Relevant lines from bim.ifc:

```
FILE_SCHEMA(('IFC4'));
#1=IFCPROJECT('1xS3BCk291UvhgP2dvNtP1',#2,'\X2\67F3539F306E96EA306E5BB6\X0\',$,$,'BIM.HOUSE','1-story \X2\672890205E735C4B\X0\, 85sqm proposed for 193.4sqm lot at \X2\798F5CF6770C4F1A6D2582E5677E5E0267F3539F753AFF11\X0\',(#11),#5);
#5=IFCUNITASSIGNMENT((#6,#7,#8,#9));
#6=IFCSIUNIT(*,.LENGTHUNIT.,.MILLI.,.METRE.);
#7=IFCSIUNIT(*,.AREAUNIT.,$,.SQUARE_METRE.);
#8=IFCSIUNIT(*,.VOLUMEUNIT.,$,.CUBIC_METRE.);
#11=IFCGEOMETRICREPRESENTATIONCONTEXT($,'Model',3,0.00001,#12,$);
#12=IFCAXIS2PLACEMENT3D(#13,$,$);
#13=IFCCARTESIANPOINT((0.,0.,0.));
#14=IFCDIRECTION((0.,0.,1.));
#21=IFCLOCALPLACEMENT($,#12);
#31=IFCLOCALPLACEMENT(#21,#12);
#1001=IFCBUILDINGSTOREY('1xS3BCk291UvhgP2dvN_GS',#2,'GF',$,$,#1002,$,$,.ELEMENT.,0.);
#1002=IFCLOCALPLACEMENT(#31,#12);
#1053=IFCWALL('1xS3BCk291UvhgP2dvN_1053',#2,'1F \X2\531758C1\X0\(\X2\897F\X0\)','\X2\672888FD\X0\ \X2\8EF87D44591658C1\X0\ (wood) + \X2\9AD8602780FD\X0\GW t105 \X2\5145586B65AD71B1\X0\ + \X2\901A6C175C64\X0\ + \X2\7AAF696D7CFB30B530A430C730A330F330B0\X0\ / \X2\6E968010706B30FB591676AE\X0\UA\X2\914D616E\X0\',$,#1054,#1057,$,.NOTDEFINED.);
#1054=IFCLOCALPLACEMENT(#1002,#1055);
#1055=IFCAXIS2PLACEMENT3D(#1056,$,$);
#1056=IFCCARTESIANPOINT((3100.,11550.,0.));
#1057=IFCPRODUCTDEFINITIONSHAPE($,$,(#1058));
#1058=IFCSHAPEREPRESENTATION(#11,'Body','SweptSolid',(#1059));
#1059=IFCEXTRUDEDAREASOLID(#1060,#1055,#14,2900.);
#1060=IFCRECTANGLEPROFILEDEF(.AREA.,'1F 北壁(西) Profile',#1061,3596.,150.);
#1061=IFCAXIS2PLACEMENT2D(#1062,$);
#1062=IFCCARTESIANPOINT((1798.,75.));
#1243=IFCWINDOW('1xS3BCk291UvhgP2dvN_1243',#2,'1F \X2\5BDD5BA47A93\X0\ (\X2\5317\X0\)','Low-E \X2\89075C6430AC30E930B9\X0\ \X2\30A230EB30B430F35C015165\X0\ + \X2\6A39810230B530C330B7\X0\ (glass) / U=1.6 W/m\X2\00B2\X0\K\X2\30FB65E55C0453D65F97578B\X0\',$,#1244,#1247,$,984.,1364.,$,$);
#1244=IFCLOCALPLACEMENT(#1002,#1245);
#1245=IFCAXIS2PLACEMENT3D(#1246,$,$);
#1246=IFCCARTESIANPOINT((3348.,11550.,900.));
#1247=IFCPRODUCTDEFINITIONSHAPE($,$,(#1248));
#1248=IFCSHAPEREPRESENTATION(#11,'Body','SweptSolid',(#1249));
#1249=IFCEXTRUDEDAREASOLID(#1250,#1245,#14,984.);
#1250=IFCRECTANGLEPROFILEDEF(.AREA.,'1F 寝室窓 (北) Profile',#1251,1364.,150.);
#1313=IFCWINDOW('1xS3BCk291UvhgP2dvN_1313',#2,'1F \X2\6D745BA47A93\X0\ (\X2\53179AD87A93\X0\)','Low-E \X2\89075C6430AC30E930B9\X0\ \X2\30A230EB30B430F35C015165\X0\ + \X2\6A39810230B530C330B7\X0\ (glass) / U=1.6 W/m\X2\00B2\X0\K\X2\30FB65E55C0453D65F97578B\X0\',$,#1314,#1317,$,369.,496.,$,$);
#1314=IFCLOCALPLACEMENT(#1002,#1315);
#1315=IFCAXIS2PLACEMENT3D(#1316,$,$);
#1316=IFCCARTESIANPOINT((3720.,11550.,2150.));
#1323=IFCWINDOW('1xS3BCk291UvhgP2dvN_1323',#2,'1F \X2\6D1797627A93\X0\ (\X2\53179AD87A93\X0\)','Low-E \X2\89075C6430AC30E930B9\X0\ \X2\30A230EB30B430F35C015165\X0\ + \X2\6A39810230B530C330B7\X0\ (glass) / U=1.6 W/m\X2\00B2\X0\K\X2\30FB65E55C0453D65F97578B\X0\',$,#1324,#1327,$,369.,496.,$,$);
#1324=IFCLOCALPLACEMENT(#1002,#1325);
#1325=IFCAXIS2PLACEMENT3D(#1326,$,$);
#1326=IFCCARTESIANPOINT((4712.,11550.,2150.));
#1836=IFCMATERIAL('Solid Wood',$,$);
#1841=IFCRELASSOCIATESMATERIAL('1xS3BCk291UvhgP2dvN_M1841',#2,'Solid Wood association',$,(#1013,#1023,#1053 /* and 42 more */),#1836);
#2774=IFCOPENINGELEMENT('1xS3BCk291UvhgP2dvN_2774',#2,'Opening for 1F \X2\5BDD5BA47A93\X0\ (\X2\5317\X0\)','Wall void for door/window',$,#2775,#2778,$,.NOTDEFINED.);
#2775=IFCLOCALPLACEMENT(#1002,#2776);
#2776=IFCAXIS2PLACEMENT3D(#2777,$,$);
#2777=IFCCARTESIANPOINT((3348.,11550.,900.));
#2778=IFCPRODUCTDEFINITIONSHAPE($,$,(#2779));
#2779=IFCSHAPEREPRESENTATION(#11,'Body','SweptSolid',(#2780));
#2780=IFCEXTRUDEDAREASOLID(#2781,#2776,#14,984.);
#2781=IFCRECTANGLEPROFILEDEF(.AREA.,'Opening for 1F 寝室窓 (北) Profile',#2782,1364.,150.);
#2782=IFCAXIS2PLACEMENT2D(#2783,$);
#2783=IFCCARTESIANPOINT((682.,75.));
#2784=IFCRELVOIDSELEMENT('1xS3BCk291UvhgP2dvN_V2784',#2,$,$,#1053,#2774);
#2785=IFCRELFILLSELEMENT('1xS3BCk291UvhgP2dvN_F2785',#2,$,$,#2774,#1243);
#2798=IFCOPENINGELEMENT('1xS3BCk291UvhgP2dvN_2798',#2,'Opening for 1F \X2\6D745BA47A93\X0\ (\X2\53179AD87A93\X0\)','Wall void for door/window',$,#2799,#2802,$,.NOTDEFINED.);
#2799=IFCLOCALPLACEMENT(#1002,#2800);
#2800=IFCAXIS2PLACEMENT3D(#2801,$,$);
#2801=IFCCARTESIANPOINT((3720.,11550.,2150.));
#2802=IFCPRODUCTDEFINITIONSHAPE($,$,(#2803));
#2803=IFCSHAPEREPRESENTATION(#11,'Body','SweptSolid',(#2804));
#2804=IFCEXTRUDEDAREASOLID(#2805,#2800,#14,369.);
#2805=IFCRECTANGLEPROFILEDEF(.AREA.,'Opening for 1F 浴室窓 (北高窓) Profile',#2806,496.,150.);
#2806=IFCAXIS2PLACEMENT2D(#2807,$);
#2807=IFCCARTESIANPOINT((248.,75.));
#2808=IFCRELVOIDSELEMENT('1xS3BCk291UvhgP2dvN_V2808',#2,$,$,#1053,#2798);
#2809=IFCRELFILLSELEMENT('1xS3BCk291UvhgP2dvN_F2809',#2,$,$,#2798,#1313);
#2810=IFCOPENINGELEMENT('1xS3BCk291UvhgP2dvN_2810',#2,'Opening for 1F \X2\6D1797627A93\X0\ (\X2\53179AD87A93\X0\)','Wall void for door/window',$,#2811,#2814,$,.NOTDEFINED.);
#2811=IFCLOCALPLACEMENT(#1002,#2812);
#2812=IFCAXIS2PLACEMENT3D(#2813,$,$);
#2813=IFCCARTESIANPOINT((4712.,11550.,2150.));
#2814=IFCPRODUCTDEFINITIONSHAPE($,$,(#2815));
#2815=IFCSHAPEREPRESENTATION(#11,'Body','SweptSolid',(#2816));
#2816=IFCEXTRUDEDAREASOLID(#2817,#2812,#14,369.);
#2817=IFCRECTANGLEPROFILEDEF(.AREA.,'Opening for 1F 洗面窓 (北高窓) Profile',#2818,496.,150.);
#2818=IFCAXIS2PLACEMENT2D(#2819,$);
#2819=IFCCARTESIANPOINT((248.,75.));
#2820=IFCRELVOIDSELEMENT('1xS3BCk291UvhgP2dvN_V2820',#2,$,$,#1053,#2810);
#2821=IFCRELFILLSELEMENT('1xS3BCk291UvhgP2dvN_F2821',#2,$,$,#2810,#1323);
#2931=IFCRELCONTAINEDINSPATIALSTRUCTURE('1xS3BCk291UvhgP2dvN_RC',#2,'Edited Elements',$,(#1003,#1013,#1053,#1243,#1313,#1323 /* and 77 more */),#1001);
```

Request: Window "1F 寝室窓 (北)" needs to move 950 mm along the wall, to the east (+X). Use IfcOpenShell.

```python
import ifcopenshell
import ifcopenshell.api.geometry
import ifcopenshell.util.placement

model = ifcopenshell.open("bim.ifc")

window = model.by_guid("1xS3BCk291UvhgP2dvN_1243")
opening = window.FillsVoids[0].RelatingOpeningElement
wall = opening.VoidsElements[0].RelatingBuildingElement

wall_matrix = ifcopenshell.util.placement.get_local_placement(wall.ObjectPlacement)
shift = wall_matrix[:3, 0] * 950.0
before = ifcopenshell.util.placement.get_local_placement(window.ObjectPlacement)[:3, 3].copy()

# The window is not placed relative to its opening, so move both.
for product in (opening, window):
    matrix = ifcopenshell.util.placement.get_local_placement(product.ObjectPlacement)
    matrix[:3, 3] += shift
    ifcopenshell.api.geometry.edit_object_placement(model, product=product, matrix=matrix, is_si=False)

after = ifcopenshell.util.placement.get_local_placement(window.ObjectPlacement)[:3, 3]
print("window moved by", (after - before).round(3) + 0.0)

model.write("bim_v2.ifc")
```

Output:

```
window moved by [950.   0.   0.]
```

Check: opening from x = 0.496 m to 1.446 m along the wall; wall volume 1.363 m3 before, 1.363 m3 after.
